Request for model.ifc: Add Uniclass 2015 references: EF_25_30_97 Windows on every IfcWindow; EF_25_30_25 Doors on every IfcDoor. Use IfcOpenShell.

First a look at what the model holds.

```python
import ifcopenshell

model = ifcopenshell.open("model.ifc")
print(model.schema)
print("classifications:", [c.Name for c in model.by_type("IfcClassification")])
for ifc_class in ("IfcDoor", "IfcRoof", "IfcStair", "IfcWall", "IfcWindow"):
    print(ifc_class, len(model.by_type(ifc_class)))
```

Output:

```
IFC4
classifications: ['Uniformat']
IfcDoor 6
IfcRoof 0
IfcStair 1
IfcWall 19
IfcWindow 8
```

```python
import ifcopenshell
import ifcopenshell.api.classification

model = ifcopenshell.open("model.ifc")

system = ifcopenshell.api.classification.add_classification(model, classification="Uniclass 2015")

codes = {
    "IfcWindow": ("EF_25_30_97", "Windows"),
    "IfcDoor": ("EF_25_30_25", "Doors"),
}
for ifc_class, (code, name) in codes.items():
    products = model.by_type(ifc_class)
    ifcopenshell.api.classification.add_reference(
        model, products=products, classification=system, identification=code, name=name
    )
    print(code, len(products))

model.write("model_updated.ifc")
```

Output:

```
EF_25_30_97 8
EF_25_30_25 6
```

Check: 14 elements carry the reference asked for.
